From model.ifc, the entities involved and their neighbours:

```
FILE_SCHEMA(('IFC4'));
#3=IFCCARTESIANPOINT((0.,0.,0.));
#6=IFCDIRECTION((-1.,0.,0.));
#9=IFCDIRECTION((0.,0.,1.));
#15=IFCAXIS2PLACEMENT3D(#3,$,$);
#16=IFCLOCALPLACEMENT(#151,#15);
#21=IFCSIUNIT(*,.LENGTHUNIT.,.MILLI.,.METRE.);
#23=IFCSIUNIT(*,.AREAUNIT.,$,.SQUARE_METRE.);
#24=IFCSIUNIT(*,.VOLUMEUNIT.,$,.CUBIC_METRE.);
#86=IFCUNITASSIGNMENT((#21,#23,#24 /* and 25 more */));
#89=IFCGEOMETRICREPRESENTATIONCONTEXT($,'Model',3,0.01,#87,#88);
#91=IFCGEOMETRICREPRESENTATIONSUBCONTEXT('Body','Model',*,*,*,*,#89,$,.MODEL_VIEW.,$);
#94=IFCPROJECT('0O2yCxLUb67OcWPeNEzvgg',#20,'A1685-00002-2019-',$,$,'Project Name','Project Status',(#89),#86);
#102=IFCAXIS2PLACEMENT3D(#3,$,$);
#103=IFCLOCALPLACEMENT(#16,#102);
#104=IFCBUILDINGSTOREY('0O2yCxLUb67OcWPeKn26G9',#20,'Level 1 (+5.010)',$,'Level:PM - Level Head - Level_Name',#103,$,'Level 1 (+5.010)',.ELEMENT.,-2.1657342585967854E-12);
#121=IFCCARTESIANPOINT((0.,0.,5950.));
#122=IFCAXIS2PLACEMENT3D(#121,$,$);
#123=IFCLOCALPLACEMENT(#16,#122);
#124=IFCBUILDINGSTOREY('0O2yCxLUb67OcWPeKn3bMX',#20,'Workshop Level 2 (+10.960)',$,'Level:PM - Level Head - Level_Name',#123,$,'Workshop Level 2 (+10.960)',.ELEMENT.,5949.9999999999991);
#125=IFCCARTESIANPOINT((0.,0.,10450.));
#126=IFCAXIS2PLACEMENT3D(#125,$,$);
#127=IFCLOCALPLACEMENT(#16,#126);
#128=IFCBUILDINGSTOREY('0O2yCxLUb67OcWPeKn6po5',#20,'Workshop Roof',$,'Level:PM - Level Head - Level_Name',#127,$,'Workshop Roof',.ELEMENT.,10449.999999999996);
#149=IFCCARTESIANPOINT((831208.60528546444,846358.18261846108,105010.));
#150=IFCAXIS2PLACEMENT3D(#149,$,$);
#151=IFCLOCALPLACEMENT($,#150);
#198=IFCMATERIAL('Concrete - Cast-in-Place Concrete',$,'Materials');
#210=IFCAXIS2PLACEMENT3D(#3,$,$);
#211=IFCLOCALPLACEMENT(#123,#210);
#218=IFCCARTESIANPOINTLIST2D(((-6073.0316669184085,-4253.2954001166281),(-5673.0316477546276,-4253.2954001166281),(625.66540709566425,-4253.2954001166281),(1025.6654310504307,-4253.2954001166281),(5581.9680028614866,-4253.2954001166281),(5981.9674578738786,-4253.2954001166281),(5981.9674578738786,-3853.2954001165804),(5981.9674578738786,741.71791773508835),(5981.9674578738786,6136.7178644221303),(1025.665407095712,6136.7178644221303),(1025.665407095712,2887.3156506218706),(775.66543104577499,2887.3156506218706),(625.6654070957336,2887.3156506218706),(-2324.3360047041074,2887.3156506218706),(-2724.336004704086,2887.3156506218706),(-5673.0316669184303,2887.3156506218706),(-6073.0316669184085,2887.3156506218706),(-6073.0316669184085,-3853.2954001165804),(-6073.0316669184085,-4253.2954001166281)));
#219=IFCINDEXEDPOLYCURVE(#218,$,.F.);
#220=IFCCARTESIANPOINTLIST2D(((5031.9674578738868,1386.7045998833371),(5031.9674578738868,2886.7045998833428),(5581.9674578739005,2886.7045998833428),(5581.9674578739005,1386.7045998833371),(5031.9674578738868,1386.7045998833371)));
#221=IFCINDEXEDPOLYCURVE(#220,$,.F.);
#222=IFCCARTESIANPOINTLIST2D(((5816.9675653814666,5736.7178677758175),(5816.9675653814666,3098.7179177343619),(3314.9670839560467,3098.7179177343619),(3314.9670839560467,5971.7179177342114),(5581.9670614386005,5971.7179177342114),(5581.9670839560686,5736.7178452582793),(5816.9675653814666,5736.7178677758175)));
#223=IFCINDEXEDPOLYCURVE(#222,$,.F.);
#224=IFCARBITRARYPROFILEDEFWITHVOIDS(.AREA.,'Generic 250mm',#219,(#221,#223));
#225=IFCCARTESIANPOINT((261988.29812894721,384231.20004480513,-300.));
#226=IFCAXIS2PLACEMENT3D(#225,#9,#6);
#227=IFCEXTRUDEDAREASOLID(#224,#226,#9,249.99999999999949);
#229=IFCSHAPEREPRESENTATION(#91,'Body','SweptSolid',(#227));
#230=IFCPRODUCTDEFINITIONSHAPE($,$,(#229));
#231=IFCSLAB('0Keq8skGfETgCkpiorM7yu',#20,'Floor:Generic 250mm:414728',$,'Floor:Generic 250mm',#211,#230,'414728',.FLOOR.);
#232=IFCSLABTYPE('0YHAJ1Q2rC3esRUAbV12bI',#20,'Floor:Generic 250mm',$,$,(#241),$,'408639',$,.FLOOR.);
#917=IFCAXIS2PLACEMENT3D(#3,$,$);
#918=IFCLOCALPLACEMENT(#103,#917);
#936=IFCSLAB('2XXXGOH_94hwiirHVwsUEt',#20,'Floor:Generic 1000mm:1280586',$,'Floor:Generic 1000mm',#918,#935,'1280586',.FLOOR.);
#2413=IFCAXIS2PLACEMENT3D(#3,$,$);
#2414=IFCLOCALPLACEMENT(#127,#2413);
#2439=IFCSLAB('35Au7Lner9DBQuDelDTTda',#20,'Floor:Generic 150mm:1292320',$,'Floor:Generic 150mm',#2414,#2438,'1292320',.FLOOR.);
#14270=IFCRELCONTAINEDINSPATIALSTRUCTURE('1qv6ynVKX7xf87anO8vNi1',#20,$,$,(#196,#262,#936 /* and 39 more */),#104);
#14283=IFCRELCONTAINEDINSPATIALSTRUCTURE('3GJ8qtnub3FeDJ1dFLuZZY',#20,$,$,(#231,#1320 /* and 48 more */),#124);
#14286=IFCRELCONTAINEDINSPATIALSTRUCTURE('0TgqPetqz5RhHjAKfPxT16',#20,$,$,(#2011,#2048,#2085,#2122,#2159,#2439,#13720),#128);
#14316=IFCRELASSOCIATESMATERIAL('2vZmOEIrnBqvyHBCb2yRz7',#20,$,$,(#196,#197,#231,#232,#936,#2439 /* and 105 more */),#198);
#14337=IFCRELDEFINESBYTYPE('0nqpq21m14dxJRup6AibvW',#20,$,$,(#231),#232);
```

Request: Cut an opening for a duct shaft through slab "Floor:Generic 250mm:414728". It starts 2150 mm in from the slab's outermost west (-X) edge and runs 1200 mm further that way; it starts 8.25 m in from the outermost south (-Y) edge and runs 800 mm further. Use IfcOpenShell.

```python
import numpy as np
import ifcopenshell
import ifcopenshell.api.feature
import ifcopenshell.api.geometry
import ifcopenshell.api.root
import ifcopenshell.geom
import ifcopenshell.util.placement
import ifcopenshell.util.representation
import ifcopenshell.util.shape
import ifcopenshell.util.unit

model = ifcopenshell.open("model.ifc")
unit_scale = ifcopenshell.util.unit.calculate_unit_scale(model)
settings = ifcopenshell.geom.settings()


def volume(element):
    """Net volume in cubic metres, openings subtracted."""
    shape = ifcopenshell.geom.create_shape(settings, element)
    return ifcopenshell.util.shape.get_volume(shape.geometry)


slab = model.by_guid("0Keq8skGfETgCkpiorM7yu")
before = volume(slab)

# Extent in the slab's own axes, in metres. The edges named are its -X and -Y sides.
slab_shape = ifcopenshell.geom.create_shape(settings, slab)
vertices = ifcopenshell.util.shape.get_vertices(slab_shape.geometry)
x_min, y_min, bottom = vertices.min(axis=0)
top = vertices[:, 2].max()

opening = ifcopenshell.api.root.create_entity(model, ifc_class="IfcOpeningElement", name="Duct shaft opening", predefined_type="OPENING")
context = ifcopenshell.util.representation.get_context(model, "Model", "Body", "MODEL_VIEW")
width, depth = 1.2, 0.8
outline = [(0.0, 0.0), (width, 0.0), (width, depth), (0.0, depth), (0.0, 0.0)]
# Overshoot both faces by 50 mm so the cut is clean.
shape = ifcopenshell.api.geometry.add_slab_representation(
    model, context=context, depth=top - bottom + 0.1, polyline=outline
)
ifcopenshell.api.geometry.assign_representation(model, product=opening, representation=shape)

matrix = ifcopenshell.util.placement.get_local_placement(slab.ObjectPlacement)
matrix[:, 3] = matrix @ np.append(np.array([x_min + 2.15, y_min + 8.25, bottom - 0.05]) / unit_scale, 1.0)
ifcopenshell.api.geometry.edit_object_placement(model, product=opening, matrix=matrix, is_si=False)
ifcopenshell.api.feature.add_feature(model, feature=opening, element=slab)

after = volume(slab)

print(f"slab volume {before:.3f} -> {after:.3f} m3")

model.write("model-out.ifc")
```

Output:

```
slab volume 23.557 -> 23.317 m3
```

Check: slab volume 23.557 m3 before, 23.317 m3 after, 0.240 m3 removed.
